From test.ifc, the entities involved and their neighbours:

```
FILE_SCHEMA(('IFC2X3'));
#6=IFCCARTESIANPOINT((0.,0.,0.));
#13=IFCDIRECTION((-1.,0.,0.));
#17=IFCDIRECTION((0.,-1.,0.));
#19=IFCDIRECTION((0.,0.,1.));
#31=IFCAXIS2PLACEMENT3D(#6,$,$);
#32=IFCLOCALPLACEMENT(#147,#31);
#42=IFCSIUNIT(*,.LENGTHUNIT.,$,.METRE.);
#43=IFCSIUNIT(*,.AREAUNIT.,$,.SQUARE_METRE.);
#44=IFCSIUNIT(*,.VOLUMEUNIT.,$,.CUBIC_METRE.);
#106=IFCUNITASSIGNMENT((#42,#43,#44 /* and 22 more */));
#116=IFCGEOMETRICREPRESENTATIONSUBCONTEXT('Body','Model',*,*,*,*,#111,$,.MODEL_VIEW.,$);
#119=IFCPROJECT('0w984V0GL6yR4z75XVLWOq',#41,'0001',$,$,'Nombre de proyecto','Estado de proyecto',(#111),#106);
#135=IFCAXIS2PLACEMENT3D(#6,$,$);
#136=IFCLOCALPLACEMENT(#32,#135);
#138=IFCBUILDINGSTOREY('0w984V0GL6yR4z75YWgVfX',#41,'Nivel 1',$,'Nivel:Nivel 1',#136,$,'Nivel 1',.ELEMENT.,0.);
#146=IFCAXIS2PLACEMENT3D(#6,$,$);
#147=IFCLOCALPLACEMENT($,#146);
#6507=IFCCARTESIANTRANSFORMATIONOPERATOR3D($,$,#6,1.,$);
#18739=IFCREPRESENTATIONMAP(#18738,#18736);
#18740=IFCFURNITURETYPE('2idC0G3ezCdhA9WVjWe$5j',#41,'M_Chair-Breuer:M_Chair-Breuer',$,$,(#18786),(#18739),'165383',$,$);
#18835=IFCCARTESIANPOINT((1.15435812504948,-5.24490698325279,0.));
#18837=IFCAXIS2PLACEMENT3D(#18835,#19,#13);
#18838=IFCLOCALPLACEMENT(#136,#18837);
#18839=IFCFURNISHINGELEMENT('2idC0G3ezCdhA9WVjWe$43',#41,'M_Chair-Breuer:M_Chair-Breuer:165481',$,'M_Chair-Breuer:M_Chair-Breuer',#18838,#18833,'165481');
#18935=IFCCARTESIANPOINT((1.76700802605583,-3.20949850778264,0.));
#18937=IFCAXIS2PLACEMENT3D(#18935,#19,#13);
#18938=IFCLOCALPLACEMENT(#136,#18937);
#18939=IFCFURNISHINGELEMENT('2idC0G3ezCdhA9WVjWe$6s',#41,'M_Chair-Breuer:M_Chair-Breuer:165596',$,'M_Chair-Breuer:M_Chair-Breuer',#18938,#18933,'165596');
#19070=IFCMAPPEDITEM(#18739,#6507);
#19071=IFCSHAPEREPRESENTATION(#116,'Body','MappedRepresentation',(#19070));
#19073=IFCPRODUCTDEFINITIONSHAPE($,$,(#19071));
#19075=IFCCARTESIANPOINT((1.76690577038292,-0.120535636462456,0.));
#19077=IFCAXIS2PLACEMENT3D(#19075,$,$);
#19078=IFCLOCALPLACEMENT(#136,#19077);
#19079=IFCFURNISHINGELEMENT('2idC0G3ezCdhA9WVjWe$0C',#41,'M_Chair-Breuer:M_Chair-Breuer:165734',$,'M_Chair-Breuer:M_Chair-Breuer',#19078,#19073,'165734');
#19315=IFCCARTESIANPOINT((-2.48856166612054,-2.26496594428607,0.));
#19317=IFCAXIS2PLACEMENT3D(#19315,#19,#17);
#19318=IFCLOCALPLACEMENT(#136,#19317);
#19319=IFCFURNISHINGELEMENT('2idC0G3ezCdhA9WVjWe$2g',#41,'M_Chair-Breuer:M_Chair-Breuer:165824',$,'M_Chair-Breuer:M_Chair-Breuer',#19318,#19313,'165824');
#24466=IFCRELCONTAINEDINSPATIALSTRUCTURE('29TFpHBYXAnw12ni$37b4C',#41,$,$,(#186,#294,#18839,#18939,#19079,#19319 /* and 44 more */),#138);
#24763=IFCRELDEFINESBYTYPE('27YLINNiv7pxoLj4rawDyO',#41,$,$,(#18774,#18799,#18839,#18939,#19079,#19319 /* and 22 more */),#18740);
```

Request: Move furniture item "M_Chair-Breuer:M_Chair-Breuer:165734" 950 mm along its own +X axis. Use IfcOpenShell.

```python
import ifcopenshell
import ifcopenshell.api.geometry
import ifcopenshell.util.placement
import ifcopenshell.util.unit

model = ifcopenshell.open("test.ifc")
unit_scale = ifcopenshell.util.unit.calculate_unit_scale(model)

item = model.by_guid("2idC0G3ezCdhA9WVjWe$0C")
matrix = ifcopenshell.util.placement.get_local_placement(item.ObjectPlacement)
matrix[:3, 3] += matrix[:3, 0] * 0.95 / unit_scale
ifcopenshell.api.geometry.edit_object_placement(model, product=item, matrix=matrix, is_si=False)

print(ifcopenshell.util.placement.get_local_placement(item.ObjectPlacement).round(3) + 0.0)

model.write("test_edited.ifc")
```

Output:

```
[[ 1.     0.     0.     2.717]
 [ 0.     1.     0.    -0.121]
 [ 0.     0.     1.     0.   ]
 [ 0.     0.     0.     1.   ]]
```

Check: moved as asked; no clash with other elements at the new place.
